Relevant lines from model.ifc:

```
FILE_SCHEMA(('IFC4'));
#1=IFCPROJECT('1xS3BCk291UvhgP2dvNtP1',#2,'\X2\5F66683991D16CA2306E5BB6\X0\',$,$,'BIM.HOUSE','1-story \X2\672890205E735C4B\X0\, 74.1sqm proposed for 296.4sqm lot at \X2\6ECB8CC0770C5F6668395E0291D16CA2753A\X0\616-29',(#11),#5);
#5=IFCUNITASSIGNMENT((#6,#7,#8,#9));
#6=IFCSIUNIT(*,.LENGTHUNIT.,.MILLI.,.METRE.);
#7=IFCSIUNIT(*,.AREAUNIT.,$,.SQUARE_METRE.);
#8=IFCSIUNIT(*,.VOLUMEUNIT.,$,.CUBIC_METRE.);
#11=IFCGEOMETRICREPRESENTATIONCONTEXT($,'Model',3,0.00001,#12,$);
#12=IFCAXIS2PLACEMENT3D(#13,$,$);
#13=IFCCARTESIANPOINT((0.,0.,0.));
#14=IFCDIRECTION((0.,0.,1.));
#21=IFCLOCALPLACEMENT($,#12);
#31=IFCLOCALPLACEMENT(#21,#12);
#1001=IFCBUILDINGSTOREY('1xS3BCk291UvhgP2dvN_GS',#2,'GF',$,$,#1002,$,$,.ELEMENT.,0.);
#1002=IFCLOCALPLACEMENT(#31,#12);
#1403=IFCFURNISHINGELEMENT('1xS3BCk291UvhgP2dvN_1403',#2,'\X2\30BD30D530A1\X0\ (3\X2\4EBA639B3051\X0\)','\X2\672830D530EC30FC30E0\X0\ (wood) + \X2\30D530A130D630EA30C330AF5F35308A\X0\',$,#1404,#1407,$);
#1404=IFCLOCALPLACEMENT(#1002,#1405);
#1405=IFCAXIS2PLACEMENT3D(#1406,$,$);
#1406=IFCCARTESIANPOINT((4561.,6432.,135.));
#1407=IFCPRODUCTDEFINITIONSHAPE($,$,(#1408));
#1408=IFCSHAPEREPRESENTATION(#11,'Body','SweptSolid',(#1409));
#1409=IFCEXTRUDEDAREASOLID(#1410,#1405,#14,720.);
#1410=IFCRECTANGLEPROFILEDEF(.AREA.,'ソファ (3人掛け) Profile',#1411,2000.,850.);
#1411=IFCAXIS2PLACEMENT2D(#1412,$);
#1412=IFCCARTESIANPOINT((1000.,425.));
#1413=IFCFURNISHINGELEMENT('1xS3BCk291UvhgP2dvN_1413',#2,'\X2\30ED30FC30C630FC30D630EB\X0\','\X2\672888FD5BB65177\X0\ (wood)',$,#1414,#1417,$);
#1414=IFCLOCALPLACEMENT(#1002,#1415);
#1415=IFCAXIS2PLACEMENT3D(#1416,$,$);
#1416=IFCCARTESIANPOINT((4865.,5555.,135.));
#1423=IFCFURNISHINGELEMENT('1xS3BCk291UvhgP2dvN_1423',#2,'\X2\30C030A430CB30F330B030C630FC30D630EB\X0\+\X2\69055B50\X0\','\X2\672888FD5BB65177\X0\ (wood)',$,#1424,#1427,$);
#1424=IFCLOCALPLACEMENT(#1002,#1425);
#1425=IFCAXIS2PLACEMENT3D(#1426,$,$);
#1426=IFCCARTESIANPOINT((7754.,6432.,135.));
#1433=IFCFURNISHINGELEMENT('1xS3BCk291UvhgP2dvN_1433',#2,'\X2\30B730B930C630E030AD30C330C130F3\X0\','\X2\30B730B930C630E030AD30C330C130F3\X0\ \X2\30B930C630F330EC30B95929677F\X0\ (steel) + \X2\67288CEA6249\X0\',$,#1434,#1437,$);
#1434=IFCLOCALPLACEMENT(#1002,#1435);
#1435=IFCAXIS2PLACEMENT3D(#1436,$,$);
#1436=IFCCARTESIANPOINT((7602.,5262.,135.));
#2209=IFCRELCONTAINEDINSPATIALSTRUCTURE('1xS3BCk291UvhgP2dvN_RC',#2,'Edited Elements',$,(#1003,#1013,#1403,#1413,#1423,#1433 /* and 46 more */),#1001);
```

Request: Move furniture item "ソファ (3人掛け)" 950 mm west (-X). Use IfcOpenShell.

```python
import ifcopenshell
import ifcopenshell.api.geometry
import ifcopenshell.util.placement

model = ifcopenshell.open("model.ifc")

item = model.by_id(1403)
matrix = ifcopenshell.util.placement.get_local_placement(item.ObjectPlacement)
matrix[0, 3] -= 950.0
ifcopenshell.api.geometry.edit_object_placement(model, product=item, matrix=matrix, is_si=False)

print(ifcopenshell.util.placement.get_local_placement(item.ObjectPlacement).round(3) + 0.0)

model.write("model-out.ifc")
```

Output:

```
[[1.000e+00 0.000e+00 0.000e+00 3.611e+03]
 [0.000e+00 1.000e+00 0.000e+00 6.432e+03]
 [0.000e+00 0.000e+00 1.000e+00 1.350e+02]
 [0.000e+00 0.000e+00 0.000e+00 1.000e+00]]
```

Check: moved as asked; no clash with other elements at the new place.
